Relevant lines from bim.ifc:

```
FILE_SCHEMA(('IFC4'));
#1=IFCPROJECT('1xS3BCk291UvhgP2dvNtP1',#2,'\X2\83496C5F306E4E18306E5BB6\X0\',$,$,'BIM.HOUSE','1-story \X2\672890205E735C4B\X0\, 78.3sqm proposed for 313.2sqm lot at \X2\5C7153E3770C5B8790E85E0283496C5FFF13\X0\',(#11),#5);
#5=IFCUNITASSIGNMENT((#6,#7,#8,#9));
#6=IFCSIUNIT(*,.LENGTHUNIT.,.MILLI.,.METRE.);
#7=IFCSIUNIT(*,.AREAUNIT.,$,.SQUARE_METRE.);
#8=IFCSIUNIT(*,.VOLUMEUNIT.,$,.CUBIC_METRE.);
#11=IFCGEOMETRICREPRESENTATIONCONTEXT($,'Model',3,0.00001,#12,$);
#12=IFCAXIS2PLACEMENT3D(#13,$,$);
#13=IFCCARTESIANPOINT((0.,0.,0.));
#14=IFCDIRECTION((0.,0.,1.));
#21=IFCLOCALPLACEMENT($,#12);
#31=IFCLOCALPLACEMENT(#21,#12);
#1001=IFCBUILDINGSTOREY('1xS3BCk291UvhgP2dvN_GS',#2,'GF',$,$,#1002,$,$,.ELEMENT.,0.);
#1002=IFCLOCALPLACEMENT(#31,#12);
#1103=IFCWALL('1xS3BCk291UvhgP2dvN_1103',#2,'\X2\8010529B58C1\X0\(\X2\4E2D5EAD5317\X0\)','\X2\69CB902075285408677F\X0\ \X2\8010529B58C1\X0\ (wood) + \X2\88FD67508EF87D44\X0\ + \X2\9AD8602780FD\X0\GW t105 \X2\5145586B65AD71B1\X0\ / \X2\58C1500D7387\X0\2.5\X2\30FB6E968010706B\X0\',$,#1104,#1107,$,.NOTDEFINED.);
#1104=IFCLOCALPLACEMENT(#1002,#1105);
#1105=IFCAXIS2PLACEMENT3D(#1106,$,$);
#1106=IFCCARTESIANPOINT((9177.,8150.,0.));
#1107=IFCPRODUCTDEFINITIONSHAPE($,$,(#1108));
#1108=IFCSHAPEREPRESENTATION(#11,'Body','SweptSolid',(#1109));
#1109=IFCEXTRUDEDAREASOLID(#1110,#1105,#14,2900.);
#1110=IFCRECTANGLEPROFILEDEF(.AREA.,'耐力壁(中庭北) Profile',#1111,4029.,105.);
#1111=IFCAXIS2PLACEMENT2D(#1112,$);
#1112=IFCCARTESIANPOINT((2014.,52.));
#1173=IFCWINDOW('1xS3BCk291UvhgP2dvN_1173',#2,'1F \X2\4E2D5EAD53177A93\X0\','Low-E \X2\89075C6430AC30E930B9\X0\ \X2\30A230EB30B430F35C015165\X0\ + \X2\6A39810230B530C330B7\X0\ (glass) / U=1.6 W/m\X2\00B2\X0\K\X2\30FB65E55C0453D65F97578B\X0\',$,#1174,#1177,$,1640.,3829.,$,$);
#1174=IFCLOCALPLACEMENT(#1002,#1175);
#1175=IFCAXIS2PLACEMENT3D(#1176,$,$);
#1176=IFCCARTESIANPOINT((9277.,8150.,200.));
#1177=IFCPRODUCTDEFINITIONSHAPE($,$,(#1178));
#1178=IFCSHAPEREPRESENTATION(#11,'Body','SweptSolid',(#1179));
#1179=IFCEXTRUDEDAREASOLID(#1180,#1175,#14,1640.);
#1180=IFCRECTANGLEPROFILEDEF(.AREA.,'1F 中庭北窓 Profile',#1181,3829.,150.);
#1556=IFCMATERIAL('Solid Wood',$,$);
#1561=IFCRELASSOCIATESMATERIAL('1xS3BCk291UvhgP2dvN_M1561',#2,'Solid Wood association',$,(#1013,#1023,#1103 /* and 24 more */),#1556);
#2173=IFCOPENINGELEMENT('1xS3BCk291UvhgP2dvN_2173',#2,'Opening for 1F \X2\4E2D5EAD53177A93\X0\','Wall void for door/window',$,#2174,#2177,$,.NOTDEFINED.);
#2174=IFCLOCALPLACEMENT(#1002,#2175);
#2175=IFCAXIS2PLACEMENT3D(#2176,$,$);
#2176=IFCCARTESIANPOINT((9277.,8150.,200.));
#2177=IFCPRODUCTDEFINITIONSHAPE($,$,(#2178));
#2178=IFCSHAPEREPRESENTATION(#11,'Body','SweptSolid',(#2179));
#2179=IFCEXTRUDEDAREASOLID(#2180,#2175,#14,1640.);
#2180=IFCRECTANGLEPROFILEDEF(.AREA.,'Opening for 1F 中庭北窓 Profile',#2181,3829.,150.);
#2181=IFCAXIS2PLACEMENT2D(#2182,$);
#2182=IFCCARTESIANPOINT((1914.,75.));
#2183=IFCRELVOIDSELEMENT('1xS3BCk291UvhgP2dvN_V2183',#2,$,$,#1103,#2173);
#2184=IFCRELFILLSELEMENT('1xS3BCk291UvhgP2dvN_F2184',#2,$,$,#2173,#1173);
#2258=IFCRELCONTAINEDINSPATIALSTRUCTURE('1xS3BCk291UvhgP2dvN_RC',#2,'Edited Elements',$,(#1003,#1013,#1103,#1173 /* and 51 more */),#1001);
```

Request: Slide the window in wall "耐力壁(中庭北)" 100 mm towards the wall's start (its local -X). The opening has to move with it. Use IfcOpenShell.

```python
import ifcopenshell
import ifcopenshell.api.geometry
import ifcopenshell.util.placement
import ifcopenshell.util.unit

model = ifcopenshell.open("bim.ifc")
unit_scale = ifcopenshell.util.unit.calculate_unit_scale(model)

window = model.by_id(1173)
opening = window.FillsVoids[0].RelatingOpeningElement
wall = opening.VoidsElements[0].RelatingBuildingElement

wall_matrix = ifcopenshell.util.placement.get_local_placement(wall.ObjectPlacement)
shift = wall_matrix[:3, 0] * -0.1 / unit_scale
before = ifcopenshell.util.placement.get_local_placement(window.ObjectPlacement)[:3, 3].copy()

# The window is not placed relative to its opening, so move both.
for product in (opening, window):
    matrix = ifcopenshell.util.placement.get_local_placement(product.ObjectPlacement)
    matrix[:3, 3] += shift
    ifcopenshell.api.geometry.edit_object_placement(model, product=product, matrix=matrix, is_si=False)

after = ifcopenshell.util.placement.get_local_placement(window.ObjectPlacement)[:3, 3]
print("window moved by", (after - before).round(3) + 0.0)

model.write("bim_v2.ifc")
```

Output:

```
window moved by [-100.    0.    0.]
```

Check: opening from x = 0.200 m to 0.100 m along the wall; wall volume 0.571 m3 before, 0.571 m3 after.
